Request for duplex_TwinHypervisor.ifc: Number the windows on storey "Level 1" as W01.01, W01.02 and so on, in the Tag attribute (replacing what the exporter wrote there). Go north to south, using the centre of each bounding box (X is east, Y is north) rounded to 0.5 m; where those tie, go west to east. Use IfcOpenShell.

First a look at what the model holds.

```python
import ifcopenshell
import ifcopenshell.util.element
import ifcopenshell.util.placement

model = ifcopenshell.open("duplex_TwinHypervisor.ifc")
print(model.schema)
storey = next(s for s in model.by_type("IfcBuildingStorey") if s.Name == "Level 1")
windows = [e for e in ifcopenshell.util.element.get_decomposition(storey) if e.is_a("IfcWindow")]
for e in sorted(windows, key=lambda e: e.id()):
    origin = ifcopenshell.util.placement.get_local_placement(e.ObjectPlacement)[:3, 3]
    print(e.id(), e.Tag, e.Name, origin.round(2) + 0.0, sep=" | ")
```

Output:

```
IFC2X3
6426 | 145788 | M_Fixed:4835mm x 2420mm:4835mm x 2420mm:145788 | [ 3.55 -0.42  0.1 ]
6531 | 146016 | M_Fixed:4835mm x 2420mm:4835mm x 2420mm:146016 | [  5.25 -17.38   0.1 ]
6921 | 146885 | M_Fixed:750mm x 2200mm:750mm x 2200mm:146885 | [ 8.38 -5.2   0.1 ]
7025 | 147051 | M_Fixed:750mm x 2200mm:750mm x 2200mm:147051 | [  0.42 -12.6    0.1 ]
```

```python
import ifcopenshell
import ifcopenshell.geom
import ifcopenshell.util.element
import ifcopenshell.util.shape

model = ifcopenshell.open("duplex_TwinHypervisor.ifc")
settings = ifcopenshell.geom.settings()
settings.set("use-world-coords", True)


def centre(element):
    shape = ifcopenshell.geom.create_shape(settings, element)
    return ifcopenshell.util.shape.get_bbox_centroid(shape.geometry)


storey = next(s for s in model.by_type("IfcBuildingStorey") if s.Name == "Level 1")
windows = [e for e in ifcopenshell.util.element.get_decomposition(storey) if e.is_a("IfcWindow")]

# Insertion points can sit at a corner or the storey origin, so sort by the geometry (in metres).
centres = {e: centre(e) for e in windows}
windows.sort(key=lambda e: (-round(centres[e][1] / 0.5), centres[e][0]))

for i, e in enumerate(windows, start=1):
    number = f"W01.{i:02d}"
    e.Tag = number
    print(e.id(), number)

model.write("duplex_TwinHypervisor-out.ifc")
```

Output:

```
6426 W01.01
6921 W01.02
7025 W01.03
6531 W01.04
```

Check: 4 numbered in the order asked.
